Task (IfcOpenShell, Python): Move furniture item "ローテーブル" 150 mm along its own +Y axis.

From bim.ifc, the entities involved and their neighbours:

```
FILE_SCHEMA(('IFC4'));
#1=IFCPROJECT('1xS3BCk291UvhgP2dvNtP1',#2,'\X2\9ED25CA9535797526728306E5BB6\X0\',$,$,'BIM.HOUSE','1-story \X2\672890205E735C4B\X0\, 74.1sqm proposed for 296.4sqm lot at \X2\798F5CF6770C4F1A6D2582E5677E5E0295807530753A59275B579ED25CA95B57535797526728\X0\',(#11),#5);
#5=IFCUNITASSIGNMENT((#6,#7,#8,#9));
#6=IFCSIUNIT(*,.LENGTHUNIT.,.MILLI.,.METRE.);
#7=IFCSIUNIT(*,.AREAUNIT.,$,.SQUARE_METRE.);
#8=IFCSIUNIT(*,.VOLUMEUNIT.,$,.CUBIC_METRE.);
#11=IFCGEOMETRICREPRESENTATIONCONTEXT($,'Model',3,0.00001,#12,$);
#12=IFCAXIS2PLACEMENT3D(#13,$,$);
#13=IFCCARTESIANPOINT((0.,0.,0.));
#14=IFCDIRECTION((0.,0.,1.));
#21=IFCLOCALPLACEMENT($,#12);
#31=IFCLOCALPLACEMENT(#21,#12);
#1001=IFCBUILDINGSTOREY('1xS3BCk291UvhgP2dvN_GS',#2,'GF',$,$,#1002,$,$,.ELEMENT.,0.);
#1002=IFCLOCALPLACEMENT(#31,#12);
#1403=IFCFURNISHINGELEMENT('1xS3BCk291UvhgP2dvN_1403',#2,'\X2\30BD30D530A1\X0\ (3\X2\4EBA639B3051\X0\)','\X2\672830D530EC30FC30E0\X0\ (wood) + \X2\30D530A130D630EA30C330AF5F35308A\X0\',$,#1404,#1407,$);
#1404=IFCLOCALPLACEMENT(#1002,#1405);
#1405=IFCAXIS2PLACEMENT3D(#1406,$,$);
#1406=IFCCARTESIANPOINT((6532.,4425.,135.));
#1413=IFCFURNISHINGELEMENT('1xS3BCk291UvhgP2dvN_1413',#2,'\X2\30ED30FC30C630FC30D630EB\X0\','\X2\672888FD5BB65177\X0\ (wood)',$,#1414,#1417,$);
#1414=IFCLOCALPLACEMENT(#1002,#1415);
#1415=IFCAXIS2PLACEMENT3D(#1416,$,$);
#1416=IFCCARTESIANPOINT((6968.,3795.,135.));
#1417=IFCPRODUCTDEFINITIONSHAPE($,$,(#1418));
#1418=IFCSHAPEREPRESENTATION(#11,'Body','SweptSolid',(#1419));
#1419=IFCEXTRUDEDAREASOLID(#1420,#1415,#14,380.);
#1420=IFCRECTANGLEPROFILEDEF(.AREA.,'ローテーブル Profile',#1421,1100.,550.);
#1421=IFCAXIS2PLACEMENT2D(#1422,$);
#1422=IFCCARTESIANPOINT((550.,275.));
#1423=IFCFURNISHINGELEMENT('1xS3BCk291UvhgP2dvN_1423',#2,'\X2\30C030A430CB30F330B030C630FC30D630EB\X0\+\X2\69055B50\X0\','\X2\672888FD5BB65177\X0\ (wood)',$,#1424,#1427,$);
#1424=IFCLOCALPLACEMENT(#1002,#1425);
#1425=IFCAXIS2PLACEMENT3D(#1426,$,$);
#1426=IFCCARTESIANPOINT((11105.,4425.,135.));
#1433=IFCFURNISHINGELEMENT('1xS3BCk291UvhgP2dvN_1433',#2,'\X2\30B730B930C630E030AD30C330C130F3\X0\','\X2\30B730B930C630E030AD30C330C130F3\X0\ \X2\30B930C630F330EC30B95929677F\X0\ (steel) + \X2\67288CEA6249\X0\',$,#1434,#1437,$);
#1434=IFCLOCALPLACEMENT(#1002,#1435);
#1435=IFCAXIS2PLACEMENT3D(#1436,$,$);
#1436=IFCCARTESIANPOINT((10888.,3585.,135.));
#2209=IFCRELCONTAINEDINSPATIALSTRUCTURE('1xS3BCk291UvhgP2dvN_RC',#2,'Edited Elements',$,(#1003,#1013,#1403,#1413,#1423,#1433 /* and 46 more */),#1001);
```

```python
import ifcopenshell
import ifcopenshell.api.geometry
import ifcopenshell.util.placement
import ifcopenshell.util.unit

model = ifcopenshell.open("bim.ifc")
unit_scale = ifcopenshell.util.unit.calculate_unit_scale(model)

item = model.by_guid("1xS3BCk291UvhgP2dvN_1413")
matrix = ifcopenshell.util.placement.get_local_placement(item.ObjectPlacement)
matrix[:3, 3] += matrix[:3, 1] * 0.15 / unit_scale
ifcopenshell.api.geometry.edit_object_placement(model, product=item, matrix=matrix, is_si=False)

print(ifcopenshell.util.placement.get_local_placement(item.ObjectPlacement).round(3) + 0.0)

model.write("bim_rev.ifc")
```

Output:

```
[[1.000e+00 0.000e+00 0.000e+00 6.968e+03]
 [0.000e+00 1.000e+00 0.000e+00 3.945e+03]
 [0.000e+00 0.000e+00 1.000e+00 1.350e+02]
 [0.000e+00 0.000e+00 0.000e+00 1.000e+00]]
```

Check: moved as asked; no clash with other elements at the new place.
